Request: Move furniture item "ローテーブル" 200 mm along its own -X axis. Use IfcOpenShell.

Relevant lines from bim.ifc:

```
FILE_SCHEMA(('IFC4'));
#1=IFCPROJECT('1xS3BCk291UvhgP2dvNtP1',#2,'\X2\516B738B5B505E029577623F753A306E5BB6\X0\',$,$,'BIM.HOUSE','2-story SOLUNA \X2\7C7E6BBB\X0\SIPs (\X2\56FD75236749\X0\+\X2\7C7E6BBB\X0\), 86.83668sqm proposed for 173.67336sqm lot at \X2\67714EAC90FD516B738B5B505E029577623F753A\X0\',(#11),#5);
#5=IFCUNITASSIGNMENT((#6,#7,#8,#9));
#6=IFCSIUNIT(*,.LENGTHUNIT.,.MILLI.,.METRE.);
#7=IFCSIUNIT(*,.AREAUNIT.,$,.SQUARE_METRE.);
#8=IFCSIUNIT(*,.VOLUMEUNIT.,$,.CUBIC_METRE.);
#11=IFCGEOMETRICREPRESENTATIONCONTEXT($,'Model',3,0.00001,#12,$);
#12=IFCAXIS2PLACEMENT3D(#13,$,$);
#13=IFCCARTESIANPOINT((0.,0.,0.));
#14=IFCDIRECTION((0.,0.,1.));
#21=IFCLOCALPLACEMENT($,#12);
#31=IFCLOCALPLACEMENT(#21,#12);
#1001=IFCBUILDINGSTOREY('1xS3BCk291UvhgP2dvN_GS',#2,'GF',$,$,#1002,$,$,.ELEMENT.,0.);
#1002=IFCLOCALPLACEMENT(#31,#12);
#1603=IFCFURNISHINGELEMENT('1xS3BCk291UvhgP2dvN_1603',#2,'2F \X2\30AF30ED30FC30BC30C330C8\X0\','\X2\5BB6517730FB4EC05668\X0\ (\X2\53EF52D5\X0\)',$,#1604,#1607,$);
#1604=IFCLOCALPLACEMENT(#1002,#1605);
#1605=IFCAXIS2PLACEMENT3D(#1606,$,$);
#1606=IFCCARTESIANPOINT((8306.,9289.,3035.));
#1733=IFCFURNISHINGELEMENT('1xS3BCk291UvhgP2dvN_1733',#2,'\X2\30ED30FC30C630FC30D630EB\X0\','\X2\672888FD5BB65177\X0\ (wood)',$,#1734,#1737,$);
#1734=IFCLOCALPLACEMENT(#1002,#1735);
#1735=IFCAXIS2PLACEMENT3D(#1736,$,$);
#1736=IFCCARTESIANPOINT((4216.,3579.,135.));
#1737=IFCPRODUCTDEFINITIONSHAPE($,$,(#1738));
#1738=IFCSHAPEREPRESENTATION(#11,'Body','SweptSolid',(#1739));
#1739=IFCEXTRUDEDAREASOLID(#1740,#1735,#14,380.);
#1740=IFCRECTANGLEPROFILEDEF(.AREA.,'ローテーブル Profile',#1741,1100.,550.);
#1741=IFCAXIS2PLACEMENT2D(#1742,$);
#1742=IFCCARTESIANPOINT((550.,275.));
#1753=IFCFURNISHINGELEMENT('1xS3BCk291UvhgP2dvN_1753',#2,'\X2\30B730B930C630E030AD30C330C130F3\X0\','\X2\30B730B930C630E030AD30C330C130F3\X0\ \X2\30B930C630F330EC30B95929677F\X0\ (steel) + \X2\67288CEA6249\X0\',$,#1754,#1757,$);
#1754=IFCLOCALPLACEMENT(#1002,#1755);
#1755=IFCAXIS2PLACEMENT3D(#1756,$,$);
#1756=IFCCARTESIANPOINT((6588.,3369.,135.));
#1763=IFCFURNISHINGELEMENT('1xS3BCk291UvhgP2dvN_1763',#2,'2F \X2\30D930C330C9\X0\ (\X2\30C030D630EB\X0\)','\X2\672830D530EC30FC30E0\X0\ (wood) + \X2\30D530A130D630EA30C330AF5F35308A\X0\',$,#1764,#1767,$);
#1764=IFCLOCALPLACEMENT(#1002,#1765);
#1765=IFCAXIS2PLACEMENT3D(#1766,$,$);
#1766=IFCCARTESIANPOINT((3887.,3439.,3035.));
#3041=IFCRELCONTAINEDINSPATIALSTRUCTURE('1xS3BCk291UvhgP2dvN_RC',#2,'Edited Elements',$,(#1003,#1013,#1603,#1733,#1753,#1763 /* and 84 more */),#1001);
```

```python
import ifcopenshell
import ifcopenshell.api.geometry
import ifcopenshell.util.placement
import ifcopenshell.util.unit

model = ifcopenshell.open("bim.ifc")
unit_scale = ifcopenshell.util.unit.calculate_unit_scale(model)

item = model.by_guid("1xS3BCk291UvhgP2dvN_1733")
matrix = ifcopenshell.util.placement.get_local_placement(item.ObjectPlacement)
matrix[:3, 3] -= matrix[:3, 0] * 0.2 / unit_scale
ifcopenshell.api.geometry.edit_object_placement(model, product=item, matrix=matrix, is_si=False)

print(ifcopenshell.util.placement.get_local_placement(item.ObjectPlacement).round(3) + 0.0)

model.write("bim_edited.ifc")
```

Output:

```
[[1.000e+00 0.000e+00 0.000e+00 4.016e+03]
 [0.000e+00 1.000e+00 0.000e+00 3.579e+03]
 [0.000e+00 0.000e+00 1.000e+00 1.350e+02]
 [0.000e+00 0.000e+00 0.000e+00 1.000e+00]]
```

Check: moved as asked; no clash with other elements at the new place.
